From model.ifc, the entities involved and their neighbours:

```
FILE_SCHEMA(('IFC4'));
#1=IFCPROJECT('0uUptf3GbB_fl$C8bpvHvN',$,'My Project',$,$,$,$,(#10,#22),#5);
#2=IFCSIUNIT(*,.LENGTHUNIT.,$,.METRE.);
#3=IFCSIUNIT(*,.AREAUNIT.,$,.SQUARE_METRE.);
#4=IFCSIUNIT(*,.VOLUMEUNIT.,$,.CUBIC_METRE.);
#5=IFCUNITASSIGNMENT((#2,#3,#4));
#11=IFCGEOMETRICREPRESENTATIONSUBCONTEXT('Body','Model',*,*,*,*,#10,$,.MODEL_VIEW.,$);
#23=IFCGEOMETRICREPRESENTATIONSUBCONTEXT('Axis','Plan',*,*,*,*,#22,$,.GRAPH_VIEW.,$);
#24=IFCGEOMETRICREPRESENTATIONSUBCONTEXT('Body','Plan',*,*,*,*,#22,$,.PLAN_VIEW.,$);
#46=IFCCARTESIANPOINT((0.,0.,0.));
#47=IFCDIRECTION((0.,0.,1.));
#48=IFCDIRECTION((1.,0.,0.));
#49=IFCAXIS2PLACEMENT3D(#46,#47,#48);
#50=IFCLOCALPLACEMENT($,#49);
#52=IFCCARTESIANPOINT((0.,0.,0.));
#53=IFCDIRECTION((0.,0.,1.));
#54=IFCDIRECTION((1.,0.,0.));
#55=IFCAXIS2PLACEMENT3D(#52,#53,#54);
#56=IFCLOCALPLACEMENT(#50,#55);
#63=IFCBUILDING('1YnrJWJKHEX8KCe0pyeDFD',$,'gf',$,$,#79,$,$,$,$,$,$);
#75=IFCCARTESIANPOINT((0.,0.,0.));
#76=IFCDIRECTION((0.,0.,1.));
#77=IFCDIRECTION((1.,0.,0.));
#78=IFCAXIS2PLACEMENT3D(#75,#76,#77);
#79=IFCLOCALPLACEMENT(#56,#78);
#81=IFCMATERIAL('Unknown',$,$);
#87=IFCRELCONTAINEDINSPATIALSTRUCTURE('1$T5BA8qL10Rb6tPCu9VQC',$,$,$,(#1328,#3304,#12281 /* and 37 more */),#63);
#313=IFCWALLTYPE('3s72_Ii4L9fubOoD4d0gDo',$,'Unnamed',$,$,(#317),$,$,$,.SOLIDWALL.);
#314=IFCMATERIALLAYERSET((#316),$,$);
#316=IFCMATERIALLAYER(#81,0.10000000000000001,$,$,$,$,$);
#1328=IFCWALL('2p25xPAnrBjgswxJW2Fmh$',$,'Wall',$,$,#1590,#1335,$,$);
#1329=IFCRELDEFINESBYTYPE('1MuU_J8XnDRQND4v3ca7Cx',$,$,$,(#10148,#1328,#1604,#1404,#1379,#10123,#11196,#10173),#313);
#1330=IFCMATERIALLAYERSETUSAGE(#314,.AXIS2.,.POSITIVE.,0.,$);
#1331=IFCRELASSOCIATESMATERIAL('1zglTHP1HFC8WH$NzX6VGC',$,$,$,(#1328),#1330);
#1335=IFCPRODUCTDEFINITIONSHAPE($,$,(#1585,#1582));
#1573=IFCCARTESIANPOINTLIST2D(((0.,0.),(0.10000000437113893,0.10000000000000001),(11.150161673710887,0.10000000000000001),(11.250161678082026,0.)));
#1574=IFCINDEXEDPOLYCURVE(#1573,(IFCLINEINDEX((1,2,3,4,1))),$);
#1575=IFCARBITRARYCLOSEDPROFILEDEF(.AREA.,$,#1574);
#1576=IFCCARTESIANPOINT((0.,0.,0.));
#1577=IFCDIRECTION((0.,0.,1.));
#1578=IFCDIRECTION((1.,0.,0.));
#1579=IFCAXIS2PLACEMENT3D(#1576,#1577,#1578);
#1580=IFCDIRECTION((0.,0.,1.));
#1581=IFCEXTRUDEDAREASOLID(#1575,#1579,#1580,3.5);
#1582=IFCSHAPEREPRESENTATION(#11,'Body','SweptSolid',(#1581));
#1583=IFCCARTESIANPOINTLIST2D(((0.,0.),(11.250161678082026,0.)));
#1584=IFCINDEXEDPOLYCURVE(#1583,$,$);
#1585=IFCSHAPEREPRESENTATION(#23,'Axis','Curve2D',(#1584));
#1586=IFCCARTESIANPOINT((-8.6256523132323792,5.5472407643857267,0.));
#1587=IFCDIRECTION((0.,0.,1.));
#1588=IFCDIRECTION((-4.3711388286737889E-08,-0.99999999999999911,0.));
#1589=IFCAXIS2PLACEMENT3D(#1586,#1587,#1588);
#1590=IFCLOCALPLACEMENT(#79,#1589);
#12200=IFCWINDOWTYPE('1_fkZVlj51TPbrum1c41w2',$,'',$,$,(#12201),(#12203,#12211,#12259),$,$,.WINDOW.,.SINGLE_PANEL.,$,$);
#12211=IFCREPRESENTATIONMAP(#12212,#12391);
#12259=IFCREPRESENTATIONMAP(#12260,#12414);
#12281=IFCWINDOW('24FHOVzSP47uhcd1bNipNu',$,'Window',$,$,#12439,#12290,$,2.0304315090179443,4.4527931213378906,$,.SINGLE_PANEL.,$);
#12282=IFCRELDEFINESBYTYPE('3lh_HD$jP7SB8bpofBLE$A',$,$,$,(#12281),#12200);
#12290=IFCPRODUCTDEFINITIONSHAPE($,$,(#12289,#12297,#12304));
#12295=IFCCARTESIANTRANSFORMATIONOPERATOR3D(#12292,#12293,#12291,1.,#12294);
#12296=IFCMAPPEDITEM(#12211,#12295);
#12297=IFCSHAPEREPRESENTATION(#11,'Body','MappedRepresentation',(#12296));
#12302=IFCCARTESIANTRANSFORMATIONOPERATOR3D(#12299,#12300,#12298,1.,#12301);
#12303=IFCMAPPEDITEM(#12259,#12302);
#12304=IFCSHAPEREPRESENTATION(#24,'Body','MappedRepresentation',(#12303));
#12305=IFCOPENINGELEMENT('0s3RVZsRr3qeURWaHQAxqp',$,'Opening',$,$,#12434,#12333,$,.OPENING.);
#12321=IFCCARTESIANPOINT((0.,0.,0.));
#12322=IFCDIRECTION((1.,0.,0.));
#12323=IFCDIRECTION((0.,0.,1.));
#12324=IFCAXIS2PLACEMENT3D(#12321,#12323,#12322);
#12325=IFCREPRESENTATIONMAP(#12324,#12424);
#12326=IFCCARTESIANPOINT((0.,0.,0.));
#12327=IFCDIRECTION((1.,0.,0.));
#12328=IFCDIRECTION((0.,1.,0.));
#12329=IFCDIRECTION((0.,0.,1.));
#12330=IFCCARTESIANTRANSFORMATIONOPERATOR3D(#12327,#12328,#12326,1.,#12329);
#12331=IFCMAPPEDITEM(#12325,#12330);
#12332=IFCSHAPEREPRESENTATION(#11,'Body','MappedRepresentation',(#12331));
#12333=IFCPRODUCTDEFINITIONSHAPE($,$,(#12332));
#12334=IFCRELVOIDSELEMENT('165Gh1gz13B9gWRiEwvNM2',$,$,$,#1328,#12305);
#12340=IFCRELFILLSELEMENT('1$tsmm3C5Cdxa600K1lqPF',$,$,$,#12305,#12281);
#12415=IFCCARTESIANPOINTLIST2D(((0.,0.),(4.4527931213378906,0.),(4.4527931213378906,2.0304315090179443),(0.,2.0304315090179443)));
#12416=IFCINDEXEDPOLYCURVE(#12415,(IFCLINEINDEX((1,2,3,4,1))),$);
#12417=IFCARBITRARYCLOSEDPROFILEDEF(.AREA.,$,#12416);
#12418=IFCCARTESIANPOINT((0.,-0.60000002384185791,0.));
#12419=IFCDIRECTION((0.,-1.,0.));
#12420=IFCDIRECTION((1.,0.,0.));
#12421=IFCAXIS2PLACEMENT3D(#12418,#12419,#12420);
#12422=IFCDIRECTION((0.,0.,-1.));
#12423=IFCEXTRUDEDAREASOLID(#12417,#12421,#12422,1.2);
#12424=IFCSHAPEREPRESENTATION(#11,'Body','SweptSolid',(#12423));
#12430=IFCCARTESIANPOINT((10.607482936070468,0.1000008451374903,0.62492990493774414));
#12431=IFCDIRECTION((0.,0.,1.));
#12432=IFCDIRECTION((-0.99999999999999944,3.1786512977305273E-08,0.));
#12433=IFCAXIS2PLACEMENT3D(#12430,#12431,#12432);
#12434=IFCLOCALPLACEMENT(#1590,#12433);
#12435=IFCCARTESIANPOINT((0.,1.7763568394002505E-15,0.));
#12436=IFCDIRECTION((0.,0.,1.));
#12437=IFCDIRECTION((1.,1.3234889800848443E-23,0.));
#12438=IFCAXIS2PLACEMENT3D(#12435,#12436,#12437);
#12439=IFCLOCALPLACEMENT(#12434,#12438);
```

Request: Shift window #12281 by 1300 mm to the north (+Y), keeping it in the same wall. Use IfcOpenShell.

```python
import ifcopenshell
import ifcopenshell.api.geometry
import ifcopenshell.util.placement
import ifcopenshell.util.unit

model = ifcopenshell.open("model.ifc")
unit_scale = ifcopenshell.util.unit.calculate_unit_scale(model)

window = model.by_guid("24FHOVzSP47uhcd1bNipNu")
opening = window.FillsVoids[0].RelatingOpeningElement
wall = opening.VoidsElements[0].RelatingBuildingElement

wall_matrix = ifcopenshell.util.placement.get_local_placement(wall.ObjectPlacement)
shift = wall_matrix[:3, 0] * -1.3 / unit_scale
before = ifcopenshell.util.placement.get_local_placement(window.ObjectPlacement)[:3, 3].copy()

# The window is placed relative to its opening, so it follows when the opening moves.
matrix = ifcopenshell.util.placement.get_local_placement(opening.ObjectPlacement)
matrix[:3, 3] += shift
ifcopenshell.api.geometry.edit_object_placement(
    model, product=opening, matrix=matrix, is_si=False, should_transform_children=True
)

after = ifcopenshell.util.placement.get_local_placement(window.ObjectPlacement)[:3, 3]
print("window moved by", (after - before).round(3) + 0.0)

model.write("model_edited.ifc")
```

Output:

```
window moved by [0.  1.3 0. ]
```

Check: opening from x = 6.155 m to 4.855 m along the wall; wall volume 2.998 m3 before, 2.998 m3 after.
